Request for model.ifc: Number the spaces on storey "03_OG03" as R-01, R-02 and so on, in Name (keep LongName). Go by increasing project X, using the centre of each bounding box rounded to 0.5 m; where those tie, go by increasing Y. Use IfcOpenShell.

First a look at what the model holds.

```python
import ifcopenshell
import ifcopenshell.util.element
import ifcopenshell.util.placement

model = ifcopenshell.open("model.ifc")
print(model.schema)
storey = next(s for s in model.by_type("IfcBuildingStorey") if s.Name == "03_OG03")
spaces = [e for e in ifcopenshell.util.element.get_decomposition(storey) if e.is_a("IfcSpace")]
for e in sorted(spaces, key=lambda e: e.id()):
    origin = ifcopenshell.util.placement.get_local_placement(e.ObjectPlacement)[:3, 3]
    print(e.id(), e.Name, e.LongName, origin.round(2) + 0.0, sep=" | ")
```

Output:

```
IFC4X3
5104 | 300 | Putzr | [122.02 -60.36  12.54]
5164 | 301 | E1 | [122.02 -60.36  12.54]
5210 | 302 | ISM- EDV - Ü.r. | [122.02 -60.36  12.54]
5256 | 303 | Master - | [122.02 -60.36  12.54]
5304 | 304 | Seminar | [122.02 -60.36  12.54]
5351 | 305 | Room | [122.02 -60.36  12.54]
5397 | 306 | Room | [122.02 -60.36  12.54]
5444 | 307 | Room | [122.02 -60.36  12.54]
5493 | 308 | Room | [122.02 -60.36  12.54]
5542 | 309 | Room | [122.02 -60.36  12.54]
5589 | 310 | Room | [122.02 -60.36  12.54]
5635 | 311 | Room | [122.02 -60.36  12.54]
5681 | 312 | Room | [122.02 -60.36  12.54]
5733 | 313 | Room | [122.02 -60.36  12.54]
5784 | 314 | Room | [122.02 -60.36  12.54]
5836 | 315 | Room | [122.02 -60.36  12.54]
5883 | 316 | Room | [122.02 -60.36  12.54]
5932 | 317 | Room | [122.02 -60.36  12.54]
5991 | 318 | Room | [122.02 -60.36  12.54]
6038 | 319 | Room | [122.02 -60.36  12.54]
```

```python
import ifcopenshell
import ifcopenshell.geom
import ifcopenshell.util.element
import ifcopenshell.util.shape

model = ifcopenshell.open("model.ifc")
settings = ifcopenshell.geom.settings()
settings.set("use-world-coords", True)


def centre(element):
    shape = ifcopenshell.geom.create_shape(settings, element)
    return ifcopenshell.util.shape.get_bbox_centroid(shape.geometry)


storey = next(s for s in model.by_type("IfcBuildingStorey") if s.Name == "03_OG03")
spaces = [e for e in ifcopenshell.util.element.get_decomposition(storey) if e.is_a("IfcSpace")]

# Insertion points can sit at a corner or the storey origin, so sort by the geometry (in metres).
centres = {e: centre(e) for e in spaces}
spaces.sort(key=lambda e: (round(centres[e][0] / 0.5), centres[e][1]))

for i, e in enumerate(spaces, start=1):
    number = f"R-{i:02d}"
    e.Name = number
    print(e.id(), number)

model.write("model_updated.ifc")
```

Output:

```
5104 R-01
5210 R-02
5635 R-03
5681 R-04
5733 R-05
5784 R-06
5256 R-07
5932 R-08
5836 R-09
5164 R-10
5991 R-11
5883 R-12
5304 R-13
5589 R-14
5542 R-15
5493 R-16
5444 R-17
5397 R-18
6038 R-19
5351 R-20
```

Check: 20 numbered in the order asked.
